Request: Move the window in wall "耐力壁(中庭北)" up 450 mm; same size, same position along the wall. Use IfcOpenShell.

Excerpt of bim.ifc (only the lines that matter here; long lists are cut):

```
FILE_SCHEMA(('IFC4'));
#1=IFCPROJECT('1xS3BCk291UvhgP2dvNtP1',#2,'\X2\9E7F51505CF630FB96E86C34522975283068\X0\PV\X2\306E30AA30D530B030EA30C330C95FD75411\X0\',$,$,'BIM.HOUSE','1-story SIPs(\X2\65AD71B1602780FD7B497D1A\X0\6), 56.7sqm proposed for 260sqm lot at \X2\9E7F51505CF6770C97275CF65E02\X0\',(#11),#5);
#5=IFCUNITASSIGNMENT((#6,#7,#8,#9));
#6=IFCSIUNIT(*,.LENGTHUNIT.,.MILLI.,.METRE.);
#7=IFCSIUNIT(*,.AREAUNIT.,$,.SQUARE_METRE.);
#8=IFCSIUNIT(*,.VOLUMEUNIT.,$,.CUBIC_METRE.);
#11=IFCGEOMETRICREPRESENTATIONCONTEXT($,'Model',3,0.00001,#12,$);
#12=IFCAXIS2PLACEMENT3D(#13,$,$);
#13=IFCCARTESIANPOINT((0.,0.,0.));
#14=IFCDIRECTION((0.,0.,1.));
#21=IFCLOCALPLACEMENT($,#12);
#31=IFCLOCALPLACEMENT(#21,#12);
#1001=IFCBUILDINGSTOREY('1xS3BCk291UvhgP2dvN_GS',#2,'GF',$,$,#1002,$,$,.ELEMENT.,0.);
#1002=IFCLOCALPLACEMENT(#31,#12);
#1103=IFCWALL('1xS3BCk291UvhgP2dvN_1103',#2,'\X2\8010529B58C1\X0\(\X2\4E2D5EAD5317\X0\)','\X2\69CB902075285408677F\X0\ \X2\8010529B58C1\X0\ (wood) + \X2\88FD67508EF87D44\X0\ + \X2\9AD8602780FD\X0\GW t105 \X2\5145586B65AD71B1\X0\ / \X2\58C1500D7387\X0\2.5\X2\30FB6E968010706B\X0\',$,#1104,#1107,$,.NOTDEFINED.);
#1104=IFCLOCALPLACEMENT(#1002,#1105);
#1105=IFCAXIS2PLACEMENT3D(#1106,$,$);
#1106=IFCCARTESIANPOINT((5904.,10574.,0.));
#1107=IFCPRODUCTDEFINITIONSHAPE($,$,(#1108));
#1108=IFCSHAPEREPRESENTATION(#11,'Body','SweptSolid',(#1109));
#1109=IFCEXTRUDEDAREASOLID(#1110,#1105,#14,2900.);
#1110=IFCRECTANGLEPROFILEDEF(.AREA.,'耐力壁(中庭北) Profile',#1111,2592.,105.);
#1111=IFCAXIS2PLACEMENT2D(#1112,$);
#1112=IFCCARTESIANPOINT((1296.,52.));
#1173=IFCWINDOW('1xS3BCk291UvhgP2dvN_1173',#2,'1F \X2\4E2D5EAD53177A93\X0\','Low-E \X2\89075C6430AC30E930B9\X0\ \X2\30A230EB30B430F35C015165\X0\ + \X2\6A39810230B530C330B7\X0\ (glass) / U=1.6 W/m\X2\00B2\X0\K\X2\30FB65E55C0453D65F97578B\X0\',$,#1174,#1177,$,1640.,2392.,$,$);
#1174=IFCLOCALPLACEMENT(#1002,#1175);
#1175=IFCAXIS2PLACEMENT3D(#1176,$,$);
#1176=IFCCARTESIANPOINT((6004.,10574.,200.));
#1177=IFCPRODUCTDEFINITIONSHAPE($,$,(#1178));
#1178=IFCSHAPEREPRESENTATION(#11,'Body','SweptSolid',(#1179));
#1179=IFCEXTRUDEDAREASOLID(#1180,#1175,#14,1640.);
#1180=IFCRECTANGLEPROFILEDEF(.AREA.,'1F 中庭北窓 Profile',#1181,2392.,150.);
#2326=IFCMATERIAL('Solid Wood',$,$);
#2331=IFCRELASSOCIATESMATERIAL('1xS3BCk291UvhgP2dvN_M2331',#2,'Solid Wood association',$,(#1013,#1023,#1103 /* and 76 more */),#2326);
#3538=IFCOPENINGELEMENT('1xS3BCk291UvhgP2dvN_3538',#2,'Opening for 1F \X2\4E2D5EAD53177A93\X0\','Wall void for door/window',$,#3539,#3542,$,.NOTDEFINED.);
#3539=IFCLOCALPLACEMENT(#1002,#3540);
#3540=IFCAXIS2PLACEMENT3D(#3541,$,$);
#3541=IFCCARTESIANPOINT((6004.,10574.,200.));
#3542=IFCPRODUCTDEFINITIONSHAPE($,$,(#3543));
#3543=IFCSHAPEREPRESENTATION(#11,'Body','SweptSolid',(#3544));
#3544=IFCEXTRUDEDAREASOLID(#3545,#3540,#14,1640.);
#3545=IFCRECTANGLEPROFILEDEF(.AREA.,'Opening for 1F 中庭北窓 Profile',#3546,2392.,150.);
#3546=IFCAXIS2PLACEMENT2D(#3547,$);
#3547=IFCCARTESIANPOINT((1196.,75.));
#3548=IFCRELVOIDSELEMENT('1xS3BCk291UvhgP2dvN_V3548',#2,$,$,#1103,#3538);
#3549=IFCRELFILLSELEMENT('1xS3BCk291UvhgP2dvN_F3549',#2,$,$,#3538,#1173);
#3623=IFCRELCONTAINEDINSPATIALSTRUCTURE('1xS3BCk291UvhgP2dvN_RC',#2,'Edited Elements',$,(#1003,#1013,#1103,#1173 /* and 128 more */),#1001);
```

```python
import numpy as np
import ifcopenshell
import ifcopenshell.api.geometry
import ifcopenshell.util.placement
import ifcopenshell.util.unit

model = ifcopenshell.open("bim.ifc")
unit_scale = ifcopenshell.util.unit.calculate_unit_scale(model)

window = model.by_guid("1xS3BCk291UvhgP2dvN_1173")
opening = window.FillsVoids[0].RelatingOpeningElement
dz = 0.45 / unit_scale

shift = np.array([0.0, 0.0, dz])
# The window is not placed relative to its opening, so move both.
for product in (opening, window):
    matrix = ifcopenshell.util.placement.get_local_placement(product.ObjectPlacement)
    matrix[:3, 3] += shift
    ifcopenshell.api.geometry.edit_object_placement(model, product=product, matrix=matrix, is_si=False)

print(f"moved by {dz * unit_scale:+.3f} m")

model.write("bim_rev.ifc")
```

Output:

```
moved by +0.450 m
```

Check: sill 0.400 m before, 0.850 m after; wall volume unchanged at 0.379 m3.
